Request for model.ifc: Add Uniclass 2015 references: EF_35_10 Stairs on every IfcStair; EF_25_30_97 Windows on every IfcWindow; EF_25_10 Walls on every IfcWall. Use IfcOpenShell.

First a look at what the model holds.

```python
import ifcopenshell

model = ifcopenshell.open("model.ifc")
print(model.schema)
print("classifications:", [c.Name for c in model.by_type("IfcClassification")])
for ifc_class in ("IfcDoor", "IfcRoof", "IfcStair", "IfcWall", "IfcWindow"):
    print(ifc_class, len(model.by_type(ifc_class)))
```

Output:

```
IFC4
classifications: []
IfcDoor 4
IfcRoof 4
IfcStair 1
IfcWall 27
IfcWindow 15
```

```python
import ifcopenshell
import ifcopenshell.api.classification

model = ifcopenshell.open("model.ifc")

system = ifcopenshell.api.classification.add_classification(model, classification="Uniclass 2015")

codes = {
    "IfcStair": ("EF_35_10", "Stairs"),
    "IfcWindow": ("EF_25_30_97", "Windows"),
    "IfcWall": ("EF_25_10", "Walls"),
}
for ifc_class, (code, name) in codes.items():
    products = model.by_type(ifc_class)
    ifcopenshell.api.classification.add_reference(
        model, products=products, classification=system, identification=code, name=name
    )
    print(code, len(products))

model.write("model_updated.ifc")
```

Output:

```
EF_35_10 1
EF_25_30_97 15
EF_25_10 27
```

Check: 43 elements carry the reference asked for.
